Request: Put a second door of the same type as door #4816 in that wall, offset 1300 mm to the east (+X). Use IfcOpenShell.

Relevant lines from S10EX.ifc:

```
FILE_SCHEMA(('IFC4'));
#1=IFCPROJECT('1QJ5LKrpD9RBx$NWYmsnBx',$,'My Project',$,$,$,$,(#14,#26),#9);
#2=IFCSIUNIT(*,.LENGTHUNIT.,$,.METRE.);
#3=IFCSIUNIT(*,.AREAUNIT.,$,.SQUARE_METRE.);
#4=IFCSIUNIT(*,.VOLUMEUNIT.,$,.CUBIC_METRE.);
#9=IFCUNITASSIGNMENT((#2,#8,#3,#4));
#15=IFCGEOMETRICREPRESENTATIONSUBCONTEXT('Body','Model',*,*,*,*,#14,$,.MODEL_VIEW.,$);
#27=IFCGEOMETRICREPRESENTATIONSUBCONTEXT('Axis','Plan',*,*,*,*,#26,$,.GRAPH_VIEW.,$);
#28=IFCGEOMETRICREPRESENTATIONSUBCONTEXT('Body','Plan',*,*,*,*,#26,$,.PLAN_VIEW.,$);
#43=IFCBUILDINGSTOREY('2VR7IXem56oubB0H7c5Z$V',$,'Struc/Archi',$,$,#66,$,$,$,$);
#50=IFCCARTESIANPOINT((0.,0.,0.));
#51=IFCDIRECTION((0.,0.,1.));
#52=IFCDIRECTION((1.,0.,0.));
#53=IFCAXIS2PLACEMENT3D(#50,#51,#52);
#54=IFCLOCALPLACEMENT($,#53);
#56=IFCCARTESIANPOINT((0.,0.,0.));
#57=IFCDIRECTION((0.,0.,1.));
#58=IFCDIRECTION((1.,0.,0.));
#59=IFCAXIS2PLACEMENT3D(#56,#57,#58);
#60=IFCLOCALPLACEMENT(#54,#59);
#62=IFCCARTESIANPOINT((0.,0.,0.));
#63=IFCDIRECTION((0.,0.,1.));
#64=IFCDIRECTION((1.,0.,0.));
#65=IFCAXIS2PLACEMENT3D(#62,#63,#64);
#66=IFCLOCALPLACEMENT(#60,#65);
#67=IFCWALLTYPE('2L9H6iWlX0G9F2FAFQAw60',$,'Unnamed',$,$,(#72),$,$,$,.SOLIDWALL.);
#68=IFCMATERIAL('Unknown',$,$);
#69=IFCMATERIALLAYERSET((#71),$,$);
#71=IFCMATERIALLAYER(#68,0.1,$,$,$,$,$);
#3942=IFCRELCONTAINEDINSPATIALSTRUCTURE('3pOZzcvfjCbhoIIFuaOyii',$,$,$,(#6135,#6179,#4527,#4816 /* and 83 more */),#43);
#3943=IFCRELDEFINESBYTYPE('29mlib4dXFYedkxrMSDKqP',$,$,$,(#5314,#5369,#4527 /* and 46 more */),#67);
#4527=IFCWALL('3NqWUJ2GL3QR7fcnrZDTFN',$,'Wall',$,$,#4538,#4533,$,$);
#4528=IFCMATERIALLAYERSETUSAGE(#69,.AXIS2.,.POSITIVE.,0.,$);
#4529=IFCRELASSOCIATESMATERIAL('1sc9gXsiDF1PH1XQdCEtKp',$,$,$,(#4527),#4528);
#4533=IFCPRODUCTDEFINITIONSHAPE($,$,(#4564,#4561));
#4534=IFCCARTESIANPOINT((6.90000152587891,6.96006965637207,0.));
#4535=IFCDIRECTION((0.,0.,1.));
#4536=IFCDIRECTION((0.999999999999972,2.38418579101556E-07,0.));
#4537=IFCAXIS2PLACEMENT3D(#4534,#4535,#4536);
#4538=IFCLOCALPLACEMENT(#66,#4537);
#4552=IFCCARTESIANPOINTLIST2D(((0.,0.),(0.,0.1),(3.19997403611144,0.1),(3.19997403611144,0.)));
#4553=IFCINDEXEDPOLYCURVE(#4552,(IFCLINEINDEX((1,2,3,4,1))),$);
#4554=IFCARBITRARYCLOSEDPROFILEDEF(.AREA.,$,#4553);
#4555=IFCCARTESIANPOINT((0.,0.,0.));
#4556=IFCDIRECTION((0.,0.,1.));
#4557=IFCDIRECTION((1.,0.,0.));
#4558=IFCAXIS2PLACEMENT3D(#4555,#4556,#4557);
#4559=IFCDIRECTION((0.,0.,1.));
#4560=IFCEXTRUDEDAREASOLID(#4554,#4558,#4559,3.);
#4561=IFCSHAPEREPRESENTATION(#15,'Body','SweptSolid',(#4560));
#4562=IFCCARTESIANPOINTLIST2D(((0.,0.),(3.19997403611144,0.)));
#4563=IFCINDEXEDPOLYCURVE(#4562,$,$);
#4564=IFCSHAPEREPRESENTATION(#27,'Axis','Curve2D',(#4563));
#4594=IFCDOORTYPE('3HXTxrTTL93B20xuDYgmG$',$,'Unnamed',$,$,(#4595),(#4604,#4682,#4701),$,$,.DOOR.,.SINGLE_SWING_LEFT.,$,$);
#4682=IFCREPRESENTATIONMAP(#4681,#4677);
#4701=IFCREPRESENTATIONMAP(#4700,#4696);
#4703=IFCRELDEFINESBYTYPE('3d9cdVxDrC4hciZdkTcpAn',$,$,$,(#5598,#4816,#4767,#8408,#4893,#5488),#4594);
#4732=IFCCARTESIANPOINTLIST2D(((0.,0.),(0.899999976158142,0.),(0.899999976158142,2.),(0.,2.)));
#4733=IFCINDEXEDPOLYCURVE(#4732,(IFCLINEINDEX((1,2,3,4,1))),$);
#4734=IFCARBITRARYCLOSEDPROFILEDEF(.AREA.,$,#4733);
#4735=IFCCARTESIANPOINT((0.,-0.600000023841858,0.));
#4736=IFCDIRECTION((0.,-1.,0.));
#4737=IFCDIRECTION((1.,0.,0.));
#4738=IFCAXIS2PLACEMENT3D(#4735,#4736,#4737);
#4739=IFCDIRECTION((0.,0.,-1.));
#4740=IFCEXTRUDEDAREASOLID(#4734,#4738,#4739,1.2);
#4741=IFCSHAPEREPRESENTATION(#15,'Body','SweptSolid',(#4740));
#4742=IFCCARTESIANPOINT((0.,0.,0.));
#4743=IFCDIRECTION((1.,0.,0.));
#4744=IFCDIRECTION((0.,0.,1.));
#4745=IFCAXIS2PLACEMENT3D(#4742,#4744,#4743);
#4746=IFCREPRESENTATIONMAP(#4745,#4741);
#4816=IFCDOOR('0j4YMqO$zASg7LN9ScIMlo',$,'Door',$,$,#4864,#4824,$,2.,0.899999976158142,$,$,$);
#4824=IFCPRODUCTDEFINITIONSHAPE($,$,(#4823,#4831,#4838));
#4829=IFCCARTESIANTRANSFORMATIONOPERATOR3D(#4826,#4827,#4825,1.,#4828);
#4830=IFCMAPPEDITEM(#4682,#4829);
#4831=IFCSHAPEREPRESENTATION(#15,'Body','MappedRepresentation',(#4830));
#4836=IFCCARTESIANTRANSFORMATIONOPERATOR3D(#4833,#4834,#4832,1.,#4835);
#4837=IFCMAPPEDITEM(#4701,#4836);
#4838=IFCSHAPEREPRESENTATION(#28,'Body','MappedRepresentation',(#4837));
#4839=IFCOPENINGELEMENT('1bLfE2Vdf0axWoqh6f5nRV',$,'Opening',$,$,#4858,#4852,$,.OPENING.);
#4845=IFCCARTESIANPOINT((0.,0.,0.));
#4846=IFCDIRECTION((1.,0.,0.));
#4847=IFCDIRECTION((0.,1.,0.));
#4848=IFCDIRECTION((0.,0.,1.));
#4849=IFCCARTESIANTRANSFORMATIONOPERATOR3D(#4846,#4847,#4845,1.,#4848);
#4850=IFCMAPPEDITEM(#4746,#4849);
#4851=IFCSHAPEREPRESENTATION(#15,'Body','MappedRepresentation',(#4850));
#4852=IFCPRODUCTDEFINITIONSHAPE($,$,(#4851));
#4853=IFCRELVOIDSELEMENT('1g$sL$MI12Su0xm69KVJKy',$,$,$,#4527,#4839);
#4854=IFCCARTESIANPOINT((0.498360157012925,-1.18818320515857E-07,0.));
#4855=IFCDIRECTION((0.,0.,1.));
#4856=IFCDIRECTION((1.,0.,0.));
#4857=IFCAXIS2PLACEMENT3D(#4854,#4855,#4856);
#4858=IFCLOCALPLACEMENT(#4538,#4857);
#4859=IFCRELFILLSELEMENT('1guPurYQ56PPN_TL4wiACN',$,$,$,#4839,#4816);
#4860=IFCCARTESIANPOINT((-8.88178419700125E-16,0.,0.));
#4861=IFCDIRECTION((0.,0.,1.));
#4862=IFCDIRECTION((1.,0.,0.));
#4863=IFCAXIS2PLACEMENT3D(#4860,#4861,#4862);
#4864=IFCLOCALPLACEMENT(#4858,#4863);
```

```python
import ifcopenshell
import ifcopenshell.api.feature
import ifcopenshell.api.geometry
import ifcopenshell.api.root
import ifcopenshell.geom
import ifcopenshell.util.element
import ifcopenshell.util.placement
import ifcopenshell.util.shape
import ifcopenshell.util.unit

model = ifcopenshell.open("S10EX.ifc")
unit_scale = ifcopenshell.util.unit.calculate_unit_scale(model)
settings = ifcopenshell.geom.settings()


def volume(element):
    """Net volume in cubic metres, openings subtracted."""
    shape = ifcopenshell.geom.create_shape(settings, element)
    return ifcopenshell.util.shape.get_volume(shape.geometry)


door = model.by_id(4816)
opening = door.FillsVoids[0].RelatingOpeningElement
wall = opening.VoidsElements[0].RelatingBuildingElement
before = volume(wall)
shift = ifcopenshell.util.placement.get_local_placement(wall.ObjectPlacement)[:3, 0] * 1.3 / unit_scale

# copy_class copies the void relationship, type, container and properties, but no geometry.
new_opening = ifcopenshell.api.root.copy_class(model, product=opening)
new_opening.Representation = ifcopenshell.util.element.copy_deep(
    model, opening.Representation, exclude=["IfcGeometricRepresentationContext", "IfcRepresentationMap"]
)
new_door = ifcopenshell.api.root.copy_class(model, product=door)
new_door.Representation = ifcopenshell.util.element.copy_deep(
    model, door.Representation, exclude=["IfcGeometricRepresentationContext", "IfcRepresentationMap"]
)
ifcopenshell.api.feature.add_filling(model, opening=new_opening, element=new_door)

for old, new in ((opening, new_opening), (door, new_door)):
    matrix = ifcopenshell.util.placement.get_local_placement(old.ObjectPlacement)
    matrix[:3, 3] += shift
    ifcopenshell.api.geometry.edit_object_placement(model, product=new, matrix=matrix, is_si=False)

after = volume(wall)

print(f"wall volume {before:.3f} -> {after:.3f} m3")

model.write("S10EX_updated.ifc")
```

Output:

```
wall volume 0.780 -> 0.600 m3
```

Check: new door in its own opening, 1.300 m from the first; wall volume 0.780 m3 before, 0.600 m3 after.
